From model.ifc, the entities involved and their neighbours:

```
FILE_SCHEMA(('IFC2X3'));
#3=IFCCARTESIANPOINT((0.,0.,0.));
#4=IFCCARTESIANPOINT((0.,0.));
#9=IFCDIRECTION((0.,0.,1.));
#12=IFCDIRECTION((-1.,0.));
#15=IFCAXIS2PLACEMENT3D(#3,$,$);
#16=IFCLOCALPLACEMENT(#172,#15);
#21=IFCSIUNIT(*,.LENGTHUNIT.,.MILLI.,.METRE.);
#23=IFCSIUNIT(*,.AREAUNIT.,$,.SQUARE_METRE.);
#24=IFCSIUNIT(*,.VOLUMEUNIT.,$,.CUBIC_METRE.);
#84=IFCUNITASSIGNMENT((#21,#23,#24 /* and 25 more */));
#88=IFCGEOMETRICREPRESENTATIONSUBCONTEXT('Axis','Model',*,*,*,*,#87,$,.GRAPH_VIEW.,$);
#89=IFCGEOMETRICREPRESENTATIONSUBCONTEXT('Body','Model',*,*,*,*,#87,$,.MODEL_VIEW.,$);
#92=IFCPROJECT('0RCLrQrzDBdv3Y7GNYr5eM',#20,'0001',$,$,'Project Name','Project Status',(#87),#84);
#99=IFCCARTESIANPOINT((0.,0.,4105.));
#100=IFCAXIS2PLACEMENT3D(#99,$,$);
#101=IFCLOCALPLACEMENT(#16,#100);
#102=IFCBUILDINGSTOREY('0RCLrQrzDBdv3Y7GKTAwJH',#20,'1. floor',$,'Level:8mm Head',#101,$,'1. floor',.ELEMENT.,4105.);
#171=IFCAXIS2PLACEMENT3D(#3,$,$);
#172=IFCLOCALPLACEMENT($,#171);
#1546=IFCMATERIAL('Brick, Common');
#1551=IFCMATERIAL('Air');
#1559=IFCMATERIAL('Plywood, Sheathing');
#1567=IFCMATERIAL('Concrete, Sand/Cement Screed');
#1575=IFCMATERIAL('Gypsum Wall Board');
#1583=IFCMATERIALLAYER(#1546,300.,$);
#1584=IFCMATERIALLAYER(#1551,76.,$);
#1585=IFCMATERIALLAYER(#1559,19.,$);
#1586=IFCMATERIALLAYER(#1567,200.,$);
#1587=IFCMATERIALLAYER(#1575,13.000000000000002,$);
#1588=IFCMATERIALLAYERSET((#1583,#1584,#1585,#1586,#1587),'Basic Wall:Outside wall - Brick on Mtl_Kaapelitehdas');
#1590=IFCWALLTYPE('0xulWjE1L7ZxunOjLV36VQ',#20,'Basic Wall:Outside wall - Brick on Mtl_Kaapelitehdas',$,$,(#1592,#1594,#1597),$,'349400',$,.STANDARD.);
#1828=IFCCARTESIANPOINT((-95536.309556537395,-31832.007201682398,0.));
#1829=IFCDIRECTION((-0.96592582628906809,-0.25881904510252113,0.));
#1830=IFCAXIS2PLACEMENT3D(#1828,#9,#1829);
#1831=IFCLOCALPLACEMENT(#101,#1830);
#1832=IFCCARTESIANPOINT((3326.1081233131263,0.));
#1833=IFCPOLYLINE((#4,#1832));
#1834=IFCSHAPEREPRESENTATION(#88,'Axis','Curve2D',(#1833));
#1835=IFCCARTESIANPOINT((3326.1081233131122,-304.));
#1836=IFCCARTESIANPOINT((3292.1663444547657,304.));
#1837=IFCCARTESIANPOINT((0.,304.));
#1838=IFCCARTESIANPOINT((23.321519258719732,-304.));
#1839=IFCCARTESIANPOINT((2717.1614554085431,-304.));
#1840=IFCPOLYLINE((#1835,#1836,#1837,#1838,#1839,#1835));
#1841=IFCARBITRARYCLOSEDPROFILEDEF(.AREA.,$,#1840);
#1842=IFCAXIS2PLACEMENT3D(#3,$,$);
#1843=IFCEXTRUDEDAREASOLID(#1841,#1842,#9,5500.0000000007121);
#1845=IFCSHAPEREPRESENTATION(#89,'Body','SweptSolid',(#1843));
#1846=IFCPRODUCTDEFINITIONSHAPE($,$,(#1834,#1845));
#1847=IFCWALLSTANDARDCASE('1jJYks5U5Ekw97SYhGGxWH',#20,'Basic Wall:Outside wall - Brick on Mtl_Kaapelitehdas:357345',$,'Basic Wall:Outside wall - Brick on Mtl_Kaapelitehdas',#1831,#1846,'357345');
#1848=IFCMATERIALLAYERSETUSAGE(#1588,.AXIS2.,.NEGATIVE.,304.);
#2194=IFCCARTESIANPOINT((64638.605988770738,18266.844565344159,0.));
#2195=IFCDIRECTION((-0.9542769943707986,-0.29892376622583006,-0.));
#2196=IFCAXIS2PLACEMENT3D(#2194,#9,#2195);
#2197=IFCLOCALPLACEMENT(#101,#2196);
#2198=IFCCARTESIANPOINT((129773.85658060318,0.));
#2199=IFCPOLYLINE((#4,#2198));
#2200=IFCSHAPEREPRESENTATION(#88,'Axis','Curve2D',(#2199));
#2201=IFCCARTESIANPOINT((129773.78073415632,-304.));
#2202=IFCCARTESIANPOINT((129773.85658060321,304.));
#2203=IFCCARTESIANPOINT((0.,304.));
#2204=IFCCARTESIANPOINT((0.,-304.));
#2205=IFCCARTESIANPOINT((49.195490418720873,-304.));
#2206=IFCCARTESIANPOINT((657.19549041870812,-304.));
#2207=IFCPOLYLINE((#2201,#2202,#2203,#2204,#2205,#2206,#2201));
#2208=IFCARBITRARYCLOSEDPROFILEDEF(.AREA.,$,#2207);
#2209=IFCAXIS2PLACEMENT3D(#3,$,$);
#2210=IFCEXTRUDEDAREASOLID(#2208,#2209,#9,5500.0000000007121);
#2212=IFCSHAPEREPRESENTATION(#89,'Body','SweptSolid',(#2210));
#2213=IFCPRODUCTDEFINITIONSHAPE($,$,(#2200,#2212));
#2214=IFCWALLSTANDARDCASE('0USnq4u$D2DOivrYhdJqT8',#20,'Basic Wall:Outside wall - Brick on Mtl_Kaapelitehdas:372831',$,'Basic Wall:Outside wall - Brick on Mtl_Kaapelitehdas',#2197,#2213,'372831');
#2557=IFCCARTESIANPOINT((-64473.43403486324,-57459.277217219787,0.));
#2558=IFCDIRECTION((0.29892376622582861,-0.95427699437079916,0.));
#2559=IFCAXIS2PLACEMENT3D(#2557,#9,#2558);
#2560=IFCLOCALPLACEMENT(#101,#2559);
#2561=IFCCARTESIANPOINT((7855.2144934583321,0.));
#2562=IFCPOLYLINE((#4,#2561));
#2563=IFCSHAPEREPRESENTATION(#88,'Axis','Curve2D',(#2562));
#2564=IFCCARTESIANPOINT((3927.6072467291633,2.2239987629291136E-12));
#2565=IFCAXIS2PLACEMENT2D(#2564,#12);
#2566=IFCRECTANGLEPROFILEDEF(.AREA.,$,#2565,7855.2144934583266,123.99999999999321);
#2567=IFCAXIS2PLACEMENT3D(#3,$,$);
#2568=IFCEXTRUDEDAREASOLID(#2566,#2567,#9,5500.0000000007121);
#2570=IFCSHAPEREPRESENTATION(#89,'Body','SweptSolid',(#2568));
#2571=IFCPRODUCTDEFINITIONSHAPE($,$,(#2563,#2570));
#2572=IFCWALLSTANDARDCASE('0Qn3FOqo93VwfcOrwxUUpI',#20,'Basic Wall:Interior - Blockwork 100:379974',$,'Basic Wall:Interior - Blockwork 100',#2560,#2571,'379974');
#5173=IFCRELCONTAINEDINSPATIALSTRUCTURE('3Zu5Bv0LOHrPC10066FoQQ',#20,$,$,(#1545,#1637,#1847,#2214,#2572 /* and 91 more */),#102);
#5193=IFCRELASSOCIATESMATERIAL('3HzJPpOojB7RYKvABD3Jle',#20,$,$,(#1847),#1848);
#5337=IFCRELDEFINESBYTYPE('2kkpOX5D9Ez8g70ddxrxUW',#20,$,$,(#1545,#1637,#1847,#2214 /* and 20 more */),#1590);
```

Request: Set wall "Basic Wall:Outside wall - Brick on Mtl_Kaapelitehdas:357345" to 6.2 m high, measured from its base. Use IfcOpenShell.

```python
import ifcopenshell
import ifcopenshell.geom
import ifcopenshell.util.representation
import ifcopenshell.util.shape
import ifcopenshell.util.unit

model = ifcopenshell.open("model.ifc")
unit_scale = ifcopenshell.util.unit.calculate_unit_scale(model)
settings = ifcopenshell.geom.settings()


def volume(element):
    """Net volume in cubic metres, openings subtracted."""
    shape = ifcopenshell.geom.create_shape(settings, element)
    return ifcopenshell.util.shape.get_volume(shape.geometry)


wall = model.by_guid("1jJYks5U5Ekw97SYhGGxWH")
before = volume(wall)

body = ifcopenshell.util.representation.get_representation(wall, "Model", "Body")
solid = body.Items[0]
old_height = solid.Depth
solid.Depth = 6.2 / unit_scale
after = volume(wall)

print(f"height {old_height:g} -> {solid.Depth:g}, volume {before:.3f} -> {after:.3f} m3")

model.write("model_v2.ifc")
```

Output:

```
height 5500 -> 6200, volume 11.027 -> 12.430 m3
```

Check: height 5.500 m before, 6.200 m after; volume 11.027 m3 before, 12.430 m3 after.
